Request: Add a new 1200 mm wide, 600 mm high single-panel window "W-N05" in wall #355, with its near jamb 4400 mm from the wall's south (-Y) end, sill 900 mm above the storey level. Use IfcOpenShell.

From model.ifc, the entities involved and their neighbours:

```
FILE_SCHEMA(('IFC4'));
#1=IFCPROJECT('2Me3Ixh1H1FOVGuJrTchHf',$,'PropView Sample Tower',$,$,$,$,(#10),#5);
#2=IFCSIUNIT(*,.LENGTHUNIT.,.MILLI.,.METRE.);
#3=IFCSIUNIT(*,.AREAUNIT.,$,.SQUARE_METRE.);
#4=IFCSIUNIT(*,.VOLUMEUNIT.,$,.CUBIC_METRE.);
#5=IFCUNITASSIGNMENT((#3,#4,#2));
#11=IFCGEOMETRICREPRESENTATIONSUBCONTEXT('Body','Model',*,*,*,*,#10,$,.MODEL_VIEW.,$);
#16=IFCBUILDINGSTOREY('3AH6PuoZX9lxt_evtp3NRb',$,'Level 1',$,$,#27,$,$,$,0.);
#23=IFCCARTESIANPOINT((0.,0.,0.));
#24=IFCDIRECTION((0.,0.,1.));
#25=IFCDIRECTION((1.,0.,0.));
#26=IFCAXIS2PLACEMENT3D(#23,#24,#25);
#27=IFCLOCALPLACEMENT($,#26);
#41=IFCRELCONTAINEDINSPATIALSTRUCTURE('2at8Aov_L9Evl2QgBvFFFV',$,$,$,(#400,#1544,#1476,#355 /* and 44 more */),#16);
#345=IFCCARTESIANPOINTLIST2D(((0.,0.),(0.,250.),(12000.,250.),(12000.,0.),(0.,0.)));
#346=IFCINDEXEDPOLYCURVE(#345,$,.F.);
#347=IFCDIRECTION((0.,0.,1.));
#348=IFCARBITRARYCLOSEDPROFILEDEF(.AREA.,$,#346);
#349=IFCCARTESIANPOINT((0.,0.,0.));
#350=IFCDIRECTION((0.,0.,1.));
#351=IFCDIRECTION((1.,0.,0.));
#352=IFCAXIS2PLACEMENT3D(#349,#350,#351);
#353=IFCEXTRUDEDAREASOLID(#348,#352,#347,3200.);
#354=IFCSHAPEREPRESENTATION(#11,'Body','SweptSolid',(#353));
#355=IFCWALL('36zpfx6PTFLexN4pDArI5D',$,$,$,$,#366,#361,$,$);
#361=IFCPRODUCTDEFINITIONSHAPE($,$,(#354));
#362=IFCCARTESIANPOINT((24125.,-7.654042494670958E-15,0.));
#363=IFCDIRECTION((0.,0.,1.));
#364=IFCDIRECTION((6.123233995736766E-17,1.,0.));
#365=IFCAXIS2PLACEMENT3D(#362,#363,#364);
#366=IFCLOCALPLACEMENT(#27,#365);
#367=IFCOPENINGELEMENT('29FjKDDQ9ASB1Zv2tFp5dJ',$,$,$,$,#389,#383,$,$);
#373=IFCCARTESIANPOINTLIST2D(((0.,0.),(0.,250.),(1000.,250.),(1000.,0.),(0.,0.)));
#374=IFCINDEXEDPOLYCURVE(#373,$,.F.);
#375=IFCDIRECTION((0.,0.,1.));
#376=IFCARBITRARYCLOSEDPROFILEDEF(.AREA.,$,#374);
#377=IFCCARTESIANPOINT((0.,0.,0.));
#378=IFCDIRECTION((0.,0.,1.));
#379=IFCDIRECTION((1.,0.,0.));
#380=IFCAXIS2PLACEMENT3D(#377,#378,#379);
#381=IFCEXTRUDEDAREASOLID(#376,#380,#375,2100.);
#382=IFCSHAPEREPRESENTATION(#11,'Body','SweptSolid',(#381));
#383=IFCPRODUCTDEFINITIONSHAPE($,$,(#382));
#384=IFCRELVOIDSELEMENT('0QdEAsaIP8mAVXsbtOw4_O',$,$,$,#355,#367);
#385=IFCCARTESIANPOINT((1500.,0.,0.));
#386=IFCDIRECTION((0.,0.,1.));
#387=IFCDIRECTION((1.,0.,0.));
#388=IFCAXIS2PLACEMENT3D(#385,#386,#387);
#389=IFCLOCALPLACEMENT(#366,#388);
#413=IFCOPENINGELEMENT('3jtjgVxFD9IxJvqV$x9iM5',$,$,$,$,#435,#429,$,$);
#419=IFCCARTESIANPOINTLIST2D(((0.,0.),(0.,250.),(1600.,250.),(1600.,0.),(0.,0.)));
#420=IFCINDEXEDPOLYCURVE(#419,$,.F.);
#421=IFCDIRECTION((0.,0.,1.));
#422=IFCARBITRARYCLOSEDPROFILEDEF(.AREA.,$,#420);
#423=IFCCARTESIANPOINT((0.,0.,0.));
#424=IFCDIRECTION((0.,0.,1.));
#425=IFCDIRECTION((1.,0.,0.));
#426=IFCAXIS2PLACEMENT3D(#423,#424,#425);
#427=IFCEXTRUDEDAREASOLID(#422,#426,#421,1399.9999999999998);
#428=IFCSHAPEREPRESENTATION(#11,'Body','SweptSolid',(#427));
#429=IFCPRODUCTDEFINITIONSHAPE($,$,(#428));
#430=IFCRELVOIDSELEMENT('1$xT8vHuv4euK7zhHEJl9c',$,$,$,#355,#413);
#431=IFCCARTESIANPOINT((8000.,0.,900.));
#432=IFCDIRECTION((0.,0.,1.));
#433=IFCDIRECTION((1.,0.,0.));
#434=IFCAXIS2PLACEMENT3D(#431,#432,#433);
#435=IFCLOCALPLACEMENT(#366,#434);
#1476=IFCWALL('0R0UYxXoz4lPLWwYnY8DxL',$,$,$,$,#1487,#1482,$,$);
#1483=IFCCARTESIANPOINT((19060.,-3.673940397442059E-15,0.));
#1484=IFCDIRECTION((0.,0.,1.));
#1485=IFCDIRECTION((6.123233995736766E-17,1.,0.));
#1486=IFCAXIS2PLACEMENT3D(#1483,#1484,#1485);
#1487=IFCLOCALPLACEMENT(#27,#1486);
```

```python
import numpy as np
import ifcopenshell
import ifcopenshell.api.feature
import ifcopenshell.api.geometry
import ifcopenshell.api.root
import ifcopenshell.api.spatial
import ifcopenshell.geom
import ifcopenshell.util.element
import ifcopenshell.util.placement
import ifcopenshell.util.representation
import ifcopenshell.util.shape
import ifcopenshell.util.unit

model = ifcopenshell.open("model.ifc")
unit_scale = ifcopenshell.util.unit.calculate_unit_scale(model)
settings = ifcopenshell.geom.settings()


def volume(element):
    """Net volume in cubic metres, openings subtracted."""
    shape = ifcopenshell.geom.create_shape(settings, element)
    return ifcopenshell.util.shape.get_volume(shape.geometry)


wall = model.by_guid("36zpfx6PTFLexN4pDArI5D")
storey = ifcopenshell.util.element.get_container(wall, ifc_class="IfcBuildingStorey")
context = ifcopenshell.util.representation.get_context(model, "Model", "Body", "MODEL_VIEW")
before = volume(wall)

width, height, from_end, sill = 1.2, 0.6, 4.4, 0.9  # metres

# The wall runs along its own X axis, and the end named is its -X end.
wall_shape = ifcopenshell.geom.create_shape(settings, wall)
x, y, z = ifcopenshell.util.shape.get_vertices(wall_shape.geometry).T
start = x.min() + from_end
face, thickness = float(y.min()), float(y.max() - y.min())
wall_matrix = ifcopenshell.util.placement.get_local_placement(wall.ObjectPlacement)
level = ifcopenshell.util.placement.get_local_placement(storey.ObjectPlacement)[2, 3]


def in_wall(x, y):
    """Placement at x, y metres in the wall's axes, at sill height."""
    matrix = wall_matrix.copy()
    matrix[:, 3] = wall_matrix @ np.array([x / unit_scale, y / unit_scale, 0.0, 1.0])
    matrix[2, 3] = level + sill / unit_scale
    return matrix


# Opening: a box that overshoots both wall faces by 50 mm.
opening = ifcopenshell.api.root.create_entity(model, ifc_class="IfcOpeningElement", predefined_type="OPENING")
box = ifcopenshell.api.geometry.add_wall_representation(
    model, context=context, length=width, height=height, thickness=thickness + 0.1
)
ifcopenshell.api.geometry.assign_representation(model, product=opening, representation=box)
ifcopenshell.api.geometry.edit_object_placement(model, product=opening, matrix=in_wall(start, face - 0.05), is_si=False)
ifcopenshell.api.feature.add_feature(model, feature=opening, element=wall)

window = ifcopenshell.api.root.create_entity(model, ifc_class="IfcWindow", name="W-N05", predefined_type="WINDOW")
window.OverallWidth, window.OverallHeight = width / unit_scale, height / unit_scale
window.PartitioningType = "SINGLE_PANEL"
body = ifcopenshell.api.geometry.add_window_representation(
    model,
    context=context,
    overall_width=window.OverallWidth,
    overall_height=window.OverallHeight,
    partition_type="SINGLE_PANEL",
)
ifcopenshell.api.geometry.assign_representation(model, product=window, representation=body)
ifcopenshell.api.spatial.assign_container(model, products=[window], relating_structure=storey)
ifcopenshell.api.feature.add_filling(model, opening=opening, element=window)

# Centre the window in the wall's thickness.
ifcopenshell.api.geometry.edit_object_placement(model, product=window, matrix=in_wall(start, face), is_si=False)
window_shape = ifcopenshell.geom.create_shape(settings, window)
depth = ifcopenshell.util.shape.get_vertices(window_shape.geometry)[:, 1]
offset = face + thickness / 2 - (depth.min() + depth.max()) / 2
ifcopenshell.api.geometry.edit_object_placement(model, product=window, matrix=in_wall(start, offset), is_si=False)

after = volume(wall)

print(f"wall volume {before:.3f} -> {after:.3f} m3")

model.write("model_edited.ifc")
```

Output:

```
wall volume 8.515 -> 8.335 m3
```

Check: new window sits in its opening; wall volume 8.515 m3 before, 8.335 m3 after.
